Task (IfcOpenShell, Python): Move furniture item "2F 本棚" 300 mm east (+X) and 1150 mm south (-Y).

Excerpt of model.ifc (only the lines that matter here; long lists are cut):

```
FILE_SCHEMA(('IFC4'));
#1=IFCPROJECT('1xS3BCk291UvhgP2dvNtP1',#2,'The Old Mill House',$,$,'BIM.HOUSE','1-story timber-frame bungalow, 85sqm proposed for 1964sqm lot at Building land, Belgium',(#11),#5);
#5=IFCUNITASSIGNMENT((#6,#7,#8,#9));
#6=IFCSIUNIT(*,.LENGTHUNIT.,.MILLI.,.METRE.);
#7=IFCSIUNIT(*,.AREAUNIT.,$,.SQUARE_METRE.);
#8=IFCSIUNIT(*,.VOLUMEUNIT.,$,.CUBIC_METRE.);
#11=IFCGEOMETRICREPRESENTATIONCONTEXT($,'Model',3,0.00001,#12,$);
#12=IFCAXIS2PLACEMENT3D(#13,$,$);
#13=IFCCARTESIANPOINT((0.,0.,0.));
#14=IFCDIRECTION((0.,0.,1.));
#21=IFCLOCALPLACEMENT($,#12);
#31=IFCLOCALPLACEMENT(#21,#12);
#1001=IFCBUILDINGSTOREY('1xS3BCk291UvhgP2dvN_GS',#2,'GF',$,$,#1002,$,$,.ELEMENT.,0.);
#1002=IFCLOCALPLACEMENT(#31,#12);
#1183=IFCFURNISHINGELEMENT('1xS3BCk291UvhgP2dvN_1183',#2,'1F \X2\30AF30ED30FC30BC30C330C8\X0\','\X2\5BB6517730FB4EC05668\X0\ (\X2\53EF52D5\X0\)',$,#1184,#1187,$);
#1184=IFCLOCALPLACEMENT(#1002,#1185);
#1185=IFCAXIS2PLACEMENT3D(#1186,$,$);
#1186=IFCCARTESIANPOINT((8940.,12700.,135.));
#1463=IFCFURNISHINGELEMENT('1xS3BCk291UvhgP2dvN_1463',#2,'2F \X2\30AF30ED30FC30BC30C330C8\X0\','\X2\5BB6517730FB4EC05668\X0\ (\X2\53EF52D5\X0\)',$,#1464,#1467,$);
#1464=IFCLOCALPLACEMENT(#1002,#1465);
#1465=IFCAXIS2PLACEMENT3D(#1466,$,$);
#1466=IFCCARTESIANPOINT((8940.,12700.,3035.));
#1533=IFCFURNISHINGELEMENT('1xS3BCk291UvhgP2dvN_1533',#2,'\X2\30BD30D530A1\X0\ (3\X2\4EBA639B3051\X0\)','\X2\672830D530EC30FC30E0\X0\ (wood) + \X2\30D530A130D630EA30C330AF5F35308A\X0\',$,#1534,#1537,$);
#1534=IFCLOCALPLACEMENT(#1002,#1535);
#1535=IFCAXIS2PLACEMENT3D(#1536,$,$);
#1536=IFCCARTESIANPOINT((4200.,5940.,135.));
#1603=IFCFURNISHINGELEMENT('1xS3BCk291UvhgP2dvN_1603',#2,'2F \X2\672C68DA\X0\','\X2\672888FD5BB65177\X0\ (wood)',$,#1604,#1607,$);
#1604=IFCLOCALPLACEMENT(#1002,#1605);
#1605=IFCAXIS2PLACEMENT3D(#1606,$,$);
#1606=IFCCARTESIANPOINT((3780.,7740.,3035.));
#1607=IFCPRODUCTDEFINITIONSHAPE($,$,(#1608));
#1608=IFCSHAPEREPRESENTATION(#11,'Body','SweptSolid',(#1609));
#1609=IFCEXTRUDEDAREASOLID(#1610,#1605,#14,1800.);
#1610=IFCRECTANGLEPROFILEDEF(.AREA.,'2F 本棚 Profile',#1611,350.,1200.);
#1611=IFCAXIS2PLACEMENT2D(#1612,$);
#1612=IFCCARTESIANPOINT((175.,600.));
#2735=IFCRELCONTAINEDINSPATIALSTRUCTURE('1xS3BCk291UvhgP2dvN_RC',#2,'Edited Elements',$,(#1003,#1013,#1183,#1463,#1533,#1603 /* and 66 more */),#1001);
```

```python
import ifcopenshell
import ifcopenshell.api.geometry
import ifcopenshell.util.placement

model = ifcopenshell.open("model.ifc")

item = model.by_id(1603)
matrix = ifcopenshell.util.placement.get_local_placement(item.ObjectPlacement)
matrix[0, 3] += 300.0
matrix[1, 3] -= 1150.0
ifcopenshell.api.geometry.edit_object_placement(model, product=item, matrix=matrix, is_si=False)

print(ifcopenshell.util.placement.get_local_placement(item.ObjectPlacement).round(3) + 0.0)

model.write("model_updated.ifc")
```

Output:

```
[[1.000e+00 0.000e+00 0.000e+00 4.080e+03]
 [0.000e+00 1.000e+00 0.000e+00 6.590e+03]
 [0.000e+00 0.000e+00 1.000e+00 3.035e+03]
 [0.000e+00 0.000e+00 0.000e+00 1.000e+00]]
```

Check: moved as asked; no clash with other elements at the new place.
